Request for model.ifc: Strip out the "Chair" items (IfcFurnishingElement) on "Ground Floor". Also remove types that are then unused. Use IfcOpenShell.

First a look at what the model holds.

```python
import ifcopenshell
import ifcopenshell.util.element

model = ifcopenshell.open("model.ifc")
print(model.schema)
storey = next(s for s in model.by_type("IfcBuildingStorey") if s.Name == "Ground Floor")
furniture = [e for e in ifcopenshell.util.element.get_decomposition(storey) if e.is_a("IfcFurnishingElement")]
seen = {}
for e in furniture:
    element_type = ifcopenshell.util.element.get_type(e)
    name = element_type.Name if element_type not in (None, e) else None
    seen[name] = seen.get(name, 0) + 1
for name, count in sorted(seen.items(), key=str):
    print(count, "x", name)
```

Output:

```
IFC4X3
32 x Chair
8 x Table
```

```python
import ifcopenshell
import ifcopenshell.api.root
import ifcopenshell.util.element

model = ifcopenshell.open("model.ifc")

storey = next(s for s in model.by_type("IfcBuildingStorey") if s.Name == "Ground Floor")
furniture = [e for e in ifcopenshell.util.element.get_decomposition(storey) if e.is_a("IfcFurnishingElement")]
targets = [e for e in furniture if (t := ifcopenshell.util.element.get_type(e)) not in (None, e) and t.Name == "Chair"]
types = {ifcopenshell.util.element.get_type(e) for e in targets} - {None, *targets}

for e in targets:
    ifcopenshell.api.root.remove_product(model, product=e)
print(len(targets), "removed")

unused = [t for t in types if not ifcopenshell.util.element.get_types(t)]
for t in unused:
    ifcopenshell.api.root.remove_product(model, product=t)
print(len(unused), "unused types removed")

model.write("model_updated.ifc")
```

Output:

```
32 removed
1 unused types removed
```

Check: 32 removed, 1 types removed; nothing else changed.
